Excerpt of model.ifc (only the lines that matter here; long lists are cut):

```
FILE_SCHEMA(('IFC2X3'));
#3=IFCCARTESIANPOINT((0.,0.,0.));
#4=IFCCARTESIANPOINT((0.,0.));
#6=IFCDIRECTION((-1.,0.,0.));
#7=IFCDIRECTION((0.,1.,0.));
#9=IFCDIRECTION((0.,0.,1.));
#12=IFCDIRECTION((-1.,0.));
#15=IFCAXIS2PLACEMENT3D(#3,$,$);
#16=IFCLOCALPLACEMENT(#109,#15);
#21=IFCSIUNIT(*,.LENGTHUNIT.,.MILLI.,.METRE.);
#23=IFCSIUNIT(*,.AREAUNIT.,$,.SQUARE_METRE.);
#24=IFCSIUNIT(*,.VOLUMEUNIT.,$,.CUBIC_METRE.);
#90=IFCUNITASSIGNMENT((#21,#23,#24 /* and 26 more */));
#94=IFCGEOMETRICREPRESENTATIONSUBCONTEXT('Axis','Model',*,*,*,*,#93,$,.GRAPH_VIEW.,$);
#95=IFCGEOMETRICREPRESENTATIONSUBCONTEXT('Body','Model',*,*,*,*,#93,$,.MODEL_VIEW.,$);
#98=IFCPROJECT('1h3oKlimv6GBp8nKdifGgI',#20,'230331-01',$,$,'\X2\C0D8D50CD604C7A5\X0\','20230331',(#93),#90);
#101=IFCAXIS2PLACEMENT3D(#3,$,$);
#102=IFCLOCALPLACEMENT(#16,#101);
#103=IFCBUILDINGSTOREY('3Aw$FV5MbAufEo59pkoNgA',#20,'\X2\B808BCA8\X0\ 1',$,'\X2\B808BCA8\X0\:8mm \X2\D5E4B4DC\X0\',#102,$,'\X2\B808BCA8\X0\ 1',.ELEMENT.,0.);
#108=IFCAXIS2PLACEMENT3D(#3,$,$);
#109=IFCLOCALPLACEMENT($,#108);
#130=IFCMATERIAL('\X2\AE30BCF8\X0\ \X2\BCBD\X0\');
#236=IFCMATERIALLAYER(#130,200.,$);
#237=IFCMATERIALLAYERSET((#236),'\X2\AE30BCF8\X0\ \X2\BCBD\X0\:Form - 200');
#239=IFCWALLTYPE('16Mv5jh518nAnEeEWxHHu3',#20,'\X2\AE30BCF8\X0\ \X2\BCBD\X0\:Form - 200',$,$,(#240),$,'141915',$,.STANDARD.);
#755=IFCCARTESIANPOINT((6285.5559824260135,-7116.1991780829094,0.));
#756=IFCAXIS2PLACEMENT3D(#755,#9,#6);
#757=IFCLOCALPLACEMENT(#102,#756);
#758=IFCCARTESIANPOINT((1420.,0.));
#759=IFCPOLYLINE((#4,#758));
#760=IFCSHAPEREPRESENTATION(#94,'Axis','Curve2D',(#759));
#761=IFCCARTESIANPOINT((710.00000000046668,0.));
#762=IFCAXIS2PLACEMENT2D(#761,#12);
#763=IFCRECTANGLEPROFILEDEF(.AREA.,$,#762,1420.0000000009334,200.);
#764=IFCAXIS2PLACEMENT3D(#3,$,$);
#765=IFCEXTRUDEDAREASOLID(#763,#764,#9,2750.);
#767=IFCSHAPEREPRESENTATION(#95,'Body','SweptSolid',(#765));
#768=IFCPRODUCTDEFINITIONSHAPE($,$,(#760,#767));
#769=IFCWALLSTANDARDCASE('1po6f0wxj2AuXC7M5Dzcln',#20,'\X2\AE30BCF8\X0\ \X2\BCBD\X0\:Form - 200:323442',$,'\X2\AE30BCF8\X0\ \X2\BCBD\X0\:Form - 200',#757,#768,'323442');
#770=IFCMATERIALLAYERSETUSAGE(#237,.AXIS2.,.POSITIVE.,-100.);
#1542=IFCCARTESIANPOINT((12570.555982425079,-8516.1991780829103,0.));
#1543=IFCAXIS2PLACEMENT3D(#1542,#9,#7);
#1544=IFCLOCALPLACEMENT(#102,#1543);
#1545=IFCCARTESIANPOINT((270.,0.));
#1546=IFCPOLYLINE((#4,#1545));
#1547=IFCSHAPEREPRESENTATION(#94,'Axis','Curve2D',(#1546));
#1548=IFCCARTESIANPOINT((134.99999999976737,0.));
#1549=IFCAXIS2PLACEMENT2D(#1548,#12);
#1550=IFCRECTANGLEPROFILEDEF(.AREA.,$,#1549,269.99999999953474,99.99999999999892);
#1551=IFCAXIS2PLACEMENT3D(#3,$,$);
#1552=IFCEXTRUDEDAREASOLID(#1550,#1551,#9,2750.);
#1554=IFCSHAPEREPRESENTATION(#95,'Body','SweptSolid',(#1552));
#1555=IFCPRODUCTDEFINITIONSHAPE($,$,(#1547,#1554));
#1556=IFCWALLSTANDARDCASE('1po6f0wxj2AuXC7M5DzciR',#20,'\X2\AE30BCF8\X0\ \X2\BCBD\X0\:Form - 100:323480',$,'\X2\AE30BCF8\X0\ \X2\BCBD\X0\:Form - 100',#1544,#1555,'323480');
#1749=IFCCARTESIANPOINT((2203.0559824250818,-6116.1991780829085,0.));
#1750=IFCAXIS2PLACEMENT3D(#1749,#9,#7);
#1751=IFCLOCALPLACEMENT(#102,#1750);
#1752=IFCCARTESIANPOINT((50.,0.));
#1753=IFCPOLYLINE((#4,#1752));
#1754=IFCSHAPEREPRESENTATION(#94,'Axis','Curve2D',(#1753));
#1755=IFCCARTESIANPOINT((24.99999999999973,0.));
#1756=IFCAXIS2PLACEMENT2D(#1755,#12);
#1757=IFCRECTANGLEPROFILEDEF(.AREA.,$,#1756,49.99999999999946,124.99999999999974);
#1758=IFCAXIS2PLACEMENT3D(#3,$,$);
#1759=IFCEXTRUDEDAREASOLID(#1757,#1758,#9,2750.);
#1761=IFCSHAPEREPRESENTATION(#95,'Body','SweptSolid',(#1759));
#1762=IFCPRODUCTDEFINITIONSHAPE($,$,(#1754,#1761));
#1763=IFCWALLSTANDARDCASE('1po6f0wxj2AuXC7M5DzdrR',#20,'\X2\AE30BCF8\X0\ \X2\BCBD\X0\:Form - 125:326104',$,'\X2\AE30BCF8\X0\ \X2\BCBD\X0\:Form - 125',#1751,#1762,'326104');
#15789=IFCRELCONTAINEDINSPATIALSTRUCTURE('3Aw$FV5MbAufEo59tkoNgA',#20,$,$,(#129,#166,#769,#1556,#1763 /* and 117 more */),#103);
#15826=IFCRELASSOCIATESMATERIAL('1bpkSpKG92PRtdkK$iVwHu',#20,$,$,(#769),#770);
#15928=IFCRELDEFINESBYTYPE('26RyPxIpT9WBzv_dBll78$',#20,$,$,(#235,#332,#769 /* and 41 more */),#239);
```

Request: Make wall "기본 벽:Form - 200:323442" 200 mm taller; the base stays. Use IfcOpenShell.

```python
import ifcopenshell
import ifcopenshell.geom
import ifcopenshell.util.representation
import ifcopenshell.util.shape
import ifcopenshell.util.unit

model = ifcopenshell.open("model.ifc")
unit_scale = ifcopenshell.util.unit.calculate_unit_scale(model)
settings = ifcopenshell.geom.settings()


def volume(element):
    """Net volume in cubic metres, openings subtracted."""
    shape = ifcopenshell.geom.create_shape(settings, element)
    return ifcopenshell.util.shape.get_volume(shape.geometry)


wall = model.by_guid("1po6f0wxj2AuXC7M5Dzcln")
before = volume(wall)

body = ifcopenshell.util.representation.get_representation(wall, "Model", "Body")
solid = body.Items[0]
old_height = solid.Depth
solid.Depth += 0.2 / unit_scale
after = volume(wall)

print(f"height {old_height:g} -> {solid.Depth:g}, volume {before:.3f} -> {after:.3f} m3")

model.write("model_edited.ifc")
```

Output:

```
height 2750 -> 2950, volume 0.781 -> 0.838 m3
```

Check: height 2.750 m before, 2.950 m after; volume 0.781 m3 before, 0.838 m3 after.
